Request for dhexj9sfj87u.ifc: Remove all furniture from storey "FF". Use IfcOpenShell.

First a look at what the model holds.

```python
import ifcopenshell
import ifcopenshell.util.element

model = ifcopenshell.open("dhexj9sfj87u.ifc")
print(model.schema)
storey = next(s for s in model.by_type("IfcBuildingStorey") if s.Name == "FF")
furniture = [e for e in ifcopenshell.util.element.get_decomposition(storey) if e.is_a("IfcFurnishingElement")]
seen = {}
for e in furniture:
    element_type = ifcopenshell.util.element.get_type(e)
    name = element_type.Name if element_type not in (None, e) else None
    seen[name] = seen.get(name, 0) + 1
for name, count in sorted(seen.items(), key=str):
    print(count, "x", name)
```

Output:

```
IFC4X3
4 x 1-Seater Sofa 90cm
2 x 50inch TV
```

```python
import ifcopenshell
import ifcopenshell.api.root
import ifcopenshell.util.element

model = ifcopenshell.open("dhexj9sfj87u.ifc")

storey = next(s for s in model.by_type("IfcBuildingStorey") if s.Name == "FF")
furniture = [e for e in ifcopenshell.util.element.get_decomposition(storey) if e.is_a("IfcFurnishingElement")]

for e in furniture:
    ifcopenshell.api.root.remove_product(model, product=e)
print(len(furniture), "removed")

model.write("dhexj9sfj87u_edited.ifc")
```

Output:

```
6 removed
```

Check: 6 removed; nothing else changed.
